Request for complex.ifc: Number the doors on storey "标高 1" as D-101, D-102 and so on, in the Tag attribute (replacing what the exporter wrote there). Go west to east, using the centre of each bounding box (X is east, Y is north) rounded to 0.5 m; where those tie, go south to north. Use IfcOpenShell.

First a look at what the model holds.

```python
import ifcopenshell
import ifcopenshell.util.element
import ifcopenshell.util.placement

model = ifcopenshell.open("complex.ifc")
print(model.schema)
storey = next(s for s in model.by_type("IfcBuildingStorey") if s.Name == "标高 1")
doors = [e for e in ifcopenshell.util.element.get_decomposition(storey) if e.is_a("IfcDoor")]
for e in sorted(doors, key=lambda e: e.id()):
    origin = ifcopenshell.util.placement.get_local_placement(e.ObjectPlacement)[:3, 3]
    print(e.id(), e.Tag, e.Name, origin.round(2) + 0.0, sep=" | ")
```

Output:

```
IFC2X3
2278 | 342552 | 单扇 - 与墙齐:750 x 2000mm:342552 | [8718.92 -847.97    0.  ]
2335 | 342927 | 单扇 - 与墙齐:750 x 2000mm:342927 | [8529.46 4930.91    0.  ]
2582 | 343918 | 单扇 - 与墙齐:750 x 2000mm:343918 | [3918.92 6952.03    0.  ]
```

```python
import ifcopenshell
import ifcopenshell.geom
import ifcopenshell.util.element
import ifcopenshell.util.shape

model = ifcopenshell.open("complex.ifc")
settings = ifcopenshell.geom.settings()
settings.set("use-world-coords", True)


def centre(element):
    shape = ifcopenshell.geom.create_shape(settings, element)
    return ifcopenshell.util.shape.get_bbox_centroid(shape.geometry)


storey = next(s for s in model.by_type("IfcBuildingStorey") if s.Name == "标高 1")
doors = [e for e in ifcopenshell.util.element.get_decomposition(storey) if e.is_a("IfcDoor")]

# Insertion points can sit at a corner or the storey origin, so sort by the geometry (in metres).
centres = {e: centre(e) for e in doors}
doors.sort(key=lambda e: (round(centres[e][0] / 0.5), centres[e][1]))

for i, e in enumerate(doors, start=1):
    number = f"D-1{i:02d}"
    e.Tag = number
    print(e.id(), number)

model.write("complex_rev.ifc")
```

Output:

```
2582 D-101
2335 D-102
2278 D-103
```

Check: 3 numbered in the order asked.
